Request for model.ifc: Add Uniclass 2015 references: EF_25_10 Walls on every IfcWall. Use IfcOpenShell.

First a look at what the model holds.

```python
import ifcopenshell

model = ifcopenshell.open("model.ifc")
print(model.schema)
print("classifications:", [c.Name for c in model.by_type("IfcClassification")])
for ifc_class in ("IfcDoor", "IfcRoof", "IfcStair", "IfcWall", "IfcWindow"):
    print(ifc_class, len(model.by_type(ifc_class)))
```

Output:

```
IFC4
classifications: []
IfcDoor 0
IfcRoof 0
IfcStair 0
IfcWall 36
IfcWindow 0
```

```python
import ifcopenshell
import ifcopenshell.api.classification

model = ifcopenshell.open("model.ifc")

system = ifcopenshell.api.classification.add_classification(model, classification="Uniclass 2015")

codes = {
    "IfcWall": ("EF_25_10", "Walls"),
}
for ifc_class, (code, name) in codes.items():
    products = model.by_type(ifc_class)
    ifcopenshell.api.classification.add_reference(
        model, products=products, classification=system, identification=code, name=name
    )
    print(code, len(products))

model.write("model-out.ifc")
```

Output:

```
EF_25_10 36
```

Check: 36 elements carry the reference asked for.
